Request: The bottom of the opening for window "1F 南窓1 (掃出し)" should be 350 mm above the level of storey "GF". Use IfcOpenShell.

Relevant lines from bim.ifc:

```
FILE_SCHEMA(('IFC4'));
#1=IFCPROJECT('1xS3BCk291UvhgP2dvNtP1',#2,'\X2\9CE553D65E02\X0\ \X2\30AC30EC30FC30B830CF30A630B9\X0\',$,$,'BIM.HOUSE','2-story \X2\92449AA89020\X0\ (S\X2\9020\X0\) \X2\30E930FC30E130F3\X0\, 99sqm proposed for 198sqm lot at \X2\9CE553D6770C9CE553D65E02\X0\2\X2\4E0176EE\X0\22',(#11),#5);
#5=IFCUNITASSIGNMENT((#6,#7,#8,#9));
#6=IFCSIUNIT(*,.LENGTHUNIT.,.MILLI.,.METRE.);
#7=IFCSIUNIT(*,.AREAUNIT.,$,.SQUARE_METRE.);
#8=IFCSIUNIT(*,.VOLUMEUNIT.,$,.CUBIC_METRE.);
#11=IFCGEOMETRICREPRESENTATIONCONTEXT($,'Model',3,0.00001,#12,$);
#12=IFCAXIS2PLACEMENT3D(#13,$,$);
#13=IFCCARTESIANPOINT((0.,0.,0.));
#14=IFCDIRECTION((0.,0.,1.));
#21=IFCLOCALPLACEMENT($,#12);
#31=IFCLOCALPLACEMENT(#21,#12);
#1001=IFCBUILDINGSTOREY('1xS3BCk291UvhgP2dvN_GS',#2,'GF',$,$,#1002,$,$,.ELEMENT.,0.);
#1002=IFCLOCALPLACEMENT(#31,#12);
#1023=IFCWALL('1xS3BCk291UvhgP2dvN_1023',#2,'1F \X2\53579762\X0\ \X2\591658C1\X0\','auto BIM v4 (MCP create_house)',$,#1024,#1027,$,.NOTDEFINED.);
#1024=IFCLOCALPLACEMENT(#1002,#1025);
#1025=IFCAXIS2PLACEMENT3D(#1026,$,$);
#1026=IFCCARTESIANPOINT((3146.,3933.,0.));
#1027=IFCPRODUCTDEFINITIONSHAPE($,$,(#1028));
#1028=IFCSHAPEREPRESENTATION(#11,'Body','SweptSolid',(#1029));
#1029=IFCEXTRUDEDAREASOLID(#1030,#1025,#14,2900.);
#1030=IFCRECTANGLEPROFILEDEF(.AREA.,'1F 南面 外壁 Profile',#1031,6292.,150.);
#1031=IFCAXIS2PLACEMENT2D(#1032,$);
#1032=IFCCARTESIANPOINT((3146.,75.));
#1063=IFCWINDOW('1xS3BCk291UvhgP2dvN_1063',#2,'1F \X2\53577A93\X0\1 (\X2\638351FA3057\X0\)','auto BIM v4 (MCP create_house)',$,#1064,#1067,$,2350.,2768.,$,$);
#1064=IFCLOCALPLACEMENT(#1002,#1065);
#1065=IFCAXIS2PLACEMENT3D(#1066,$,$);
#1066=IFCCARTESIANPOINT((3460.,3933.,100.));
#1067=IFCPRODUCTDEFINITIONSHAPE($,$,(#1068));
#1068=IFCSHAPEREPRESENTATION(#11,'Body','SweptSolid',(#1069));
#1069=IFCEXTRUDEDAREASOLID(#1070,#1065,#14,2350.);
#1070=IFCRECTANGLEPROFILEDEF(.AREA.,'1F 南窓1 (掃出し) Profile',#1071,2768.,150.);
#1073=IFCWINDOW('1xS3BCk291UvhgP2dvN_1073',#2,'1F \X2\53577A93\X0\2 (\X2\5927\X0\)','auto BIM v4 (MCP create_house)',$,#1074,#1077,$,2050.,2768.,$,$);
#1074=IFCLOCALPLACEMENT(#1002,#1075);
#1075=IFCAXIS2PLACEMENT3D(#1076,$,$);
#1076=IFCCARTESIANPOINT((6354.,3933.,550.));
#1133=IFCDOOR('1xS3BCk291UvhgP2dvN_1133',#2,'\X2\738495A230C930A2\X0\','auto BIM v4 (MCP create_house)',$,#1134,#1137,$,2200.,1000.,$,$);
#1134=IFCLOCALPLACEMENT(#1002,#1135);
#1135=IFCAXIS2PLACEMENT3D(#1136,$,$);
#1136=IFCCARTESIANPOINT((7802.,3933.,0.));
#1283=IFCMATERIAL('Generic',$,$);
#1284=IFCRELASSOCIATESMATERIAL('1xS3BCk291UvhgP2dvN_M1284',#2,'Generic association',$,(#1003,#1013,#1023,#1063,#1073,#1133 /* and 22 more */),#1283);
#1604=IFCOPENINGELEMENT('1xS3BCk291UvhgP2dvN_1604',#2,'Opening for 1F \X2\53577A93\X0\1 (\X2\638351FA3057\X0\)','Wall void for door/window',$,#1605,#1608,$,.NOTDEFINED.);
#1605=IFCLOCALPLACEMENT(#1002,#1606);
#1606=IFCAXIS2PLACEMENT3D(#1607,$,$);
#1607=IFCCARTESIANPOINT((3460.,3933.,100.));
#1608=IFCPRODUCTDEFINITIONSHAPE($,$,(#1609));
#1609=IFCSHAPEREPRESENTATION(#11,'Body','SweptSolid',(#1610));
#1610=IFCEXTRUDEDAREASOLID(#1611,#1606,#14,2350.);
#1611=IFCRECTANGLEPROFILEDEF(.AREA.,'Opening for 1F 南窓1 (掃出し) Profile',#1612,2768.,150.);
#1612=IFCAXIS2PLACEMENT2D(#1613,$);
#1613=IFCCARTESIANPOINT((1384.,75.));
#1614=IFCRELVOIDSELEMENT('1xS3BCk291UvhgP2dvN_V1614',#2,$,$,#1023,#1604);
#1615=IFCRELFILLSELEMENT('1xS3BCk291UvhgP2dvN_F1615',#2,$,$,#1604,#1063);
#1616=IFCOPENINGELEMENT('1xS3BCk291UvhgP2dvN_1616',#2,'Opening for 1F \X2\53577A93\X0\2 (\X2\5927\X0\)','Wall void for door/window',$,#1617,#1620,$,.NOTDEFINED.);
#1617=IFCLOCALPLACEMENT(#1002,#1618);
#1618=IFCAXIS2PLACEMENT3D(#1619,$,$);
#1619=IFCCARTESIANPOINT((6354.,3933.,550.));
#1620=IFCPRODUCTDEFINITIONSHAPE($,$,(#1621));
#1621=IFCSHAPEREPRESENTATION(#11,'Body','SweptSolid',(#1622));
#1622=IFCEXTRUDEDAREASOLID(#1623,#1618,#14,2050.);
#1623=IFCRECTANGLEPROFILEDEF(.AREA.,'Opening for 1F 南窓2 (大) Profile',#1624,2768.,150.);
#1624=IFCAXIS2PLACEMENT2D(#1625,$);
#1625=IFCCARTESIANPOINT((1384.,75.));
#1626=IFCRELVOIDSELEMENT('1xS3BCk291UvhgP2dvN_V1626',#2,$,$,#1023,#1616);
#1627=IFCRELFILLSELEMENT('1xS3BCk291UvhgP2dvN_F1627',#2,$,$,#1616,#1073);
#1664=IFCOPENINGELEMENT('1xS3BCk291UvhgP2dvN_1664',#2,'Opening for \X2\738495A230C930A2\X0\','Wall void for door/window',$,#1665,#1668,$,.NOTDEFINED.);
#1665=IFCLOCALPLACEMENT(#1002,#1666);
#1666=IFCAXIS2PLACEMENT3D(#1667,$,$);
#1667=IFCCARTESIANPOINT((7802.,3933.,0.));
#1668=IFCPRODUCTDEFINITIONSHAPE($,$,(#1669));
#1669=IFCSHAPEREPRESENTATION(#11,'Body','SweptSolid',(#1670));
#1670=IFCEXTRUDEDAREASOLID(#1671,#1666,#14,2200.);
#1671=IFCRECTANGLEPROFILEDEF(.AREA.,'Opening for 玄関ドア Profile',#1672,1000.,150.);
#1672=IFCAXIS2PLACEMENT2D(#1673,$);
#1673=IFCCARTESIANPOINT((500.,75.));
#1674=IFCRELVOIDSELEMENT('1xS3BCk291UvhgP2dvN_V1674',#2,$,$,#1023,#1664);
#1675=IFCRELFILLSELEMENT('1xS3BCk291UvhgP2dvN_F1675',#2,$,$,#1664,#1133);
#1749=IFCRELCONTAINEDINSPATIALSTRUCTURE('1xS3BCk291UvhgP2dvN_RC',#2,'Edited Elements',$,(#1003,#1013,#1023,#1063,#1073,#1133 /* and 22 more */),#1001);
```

```python
import numpy as np
import ifcopenshell
import ifcopenshell.api.geometry
import ifcopenshell.geom
import ifcopenshell.util.element
import ifcopenshell.util.placement
import ifcopenshell.util.shape
import ifcopenshell.util.unit

model = ifcopenshell.open("bim.ifc")
unit_scale = ifcopenshell.util.unit.calculate_unit_scale(model)

window = model.by_guid("1xS3BCk291UvhgP2dvN_1063")
opening = window.FillsVoids[0].RelatingOpeningElement
storey = ifcopenshell.util.element.get_container(window, ifc_class="IfcBuildingStorey")
level = ifcopenshell.util.placement.get_local_placement(storey.ObjectPlacement)[2, 3]

# The opening's origin need not be at the sill, so measure its lowest point.
shape = ifcopenshell.geom.create_shape(ifcopenshell.geom.settings(), opening)
bottom = ifcopenshell.util.shape.get_shape_bottom_elevation(shape, shape.geometry) / unit_scale
dz = level + 0.35 / unit_scale - bottom

shift = np.array([0.0, 0.0, dz])
# The window is not placed relative to its opening, so move both.
for product in (opening, window):
    matrix = ifcopenshell.util.placement.get_local_placement(product.ObjectPlacement)
    matrix[:3, 3] += shift
    ifcopenshell.api.geometry.edit_object_placement(model, product=product, matrix=matrix, is_si=False)

print(f"moved by {dz * unit_scale:+.3f} m")

model.write("bim-out.ifc")
```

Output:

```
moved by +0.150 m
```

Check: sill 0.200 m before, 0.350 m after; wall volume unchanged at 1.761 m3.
